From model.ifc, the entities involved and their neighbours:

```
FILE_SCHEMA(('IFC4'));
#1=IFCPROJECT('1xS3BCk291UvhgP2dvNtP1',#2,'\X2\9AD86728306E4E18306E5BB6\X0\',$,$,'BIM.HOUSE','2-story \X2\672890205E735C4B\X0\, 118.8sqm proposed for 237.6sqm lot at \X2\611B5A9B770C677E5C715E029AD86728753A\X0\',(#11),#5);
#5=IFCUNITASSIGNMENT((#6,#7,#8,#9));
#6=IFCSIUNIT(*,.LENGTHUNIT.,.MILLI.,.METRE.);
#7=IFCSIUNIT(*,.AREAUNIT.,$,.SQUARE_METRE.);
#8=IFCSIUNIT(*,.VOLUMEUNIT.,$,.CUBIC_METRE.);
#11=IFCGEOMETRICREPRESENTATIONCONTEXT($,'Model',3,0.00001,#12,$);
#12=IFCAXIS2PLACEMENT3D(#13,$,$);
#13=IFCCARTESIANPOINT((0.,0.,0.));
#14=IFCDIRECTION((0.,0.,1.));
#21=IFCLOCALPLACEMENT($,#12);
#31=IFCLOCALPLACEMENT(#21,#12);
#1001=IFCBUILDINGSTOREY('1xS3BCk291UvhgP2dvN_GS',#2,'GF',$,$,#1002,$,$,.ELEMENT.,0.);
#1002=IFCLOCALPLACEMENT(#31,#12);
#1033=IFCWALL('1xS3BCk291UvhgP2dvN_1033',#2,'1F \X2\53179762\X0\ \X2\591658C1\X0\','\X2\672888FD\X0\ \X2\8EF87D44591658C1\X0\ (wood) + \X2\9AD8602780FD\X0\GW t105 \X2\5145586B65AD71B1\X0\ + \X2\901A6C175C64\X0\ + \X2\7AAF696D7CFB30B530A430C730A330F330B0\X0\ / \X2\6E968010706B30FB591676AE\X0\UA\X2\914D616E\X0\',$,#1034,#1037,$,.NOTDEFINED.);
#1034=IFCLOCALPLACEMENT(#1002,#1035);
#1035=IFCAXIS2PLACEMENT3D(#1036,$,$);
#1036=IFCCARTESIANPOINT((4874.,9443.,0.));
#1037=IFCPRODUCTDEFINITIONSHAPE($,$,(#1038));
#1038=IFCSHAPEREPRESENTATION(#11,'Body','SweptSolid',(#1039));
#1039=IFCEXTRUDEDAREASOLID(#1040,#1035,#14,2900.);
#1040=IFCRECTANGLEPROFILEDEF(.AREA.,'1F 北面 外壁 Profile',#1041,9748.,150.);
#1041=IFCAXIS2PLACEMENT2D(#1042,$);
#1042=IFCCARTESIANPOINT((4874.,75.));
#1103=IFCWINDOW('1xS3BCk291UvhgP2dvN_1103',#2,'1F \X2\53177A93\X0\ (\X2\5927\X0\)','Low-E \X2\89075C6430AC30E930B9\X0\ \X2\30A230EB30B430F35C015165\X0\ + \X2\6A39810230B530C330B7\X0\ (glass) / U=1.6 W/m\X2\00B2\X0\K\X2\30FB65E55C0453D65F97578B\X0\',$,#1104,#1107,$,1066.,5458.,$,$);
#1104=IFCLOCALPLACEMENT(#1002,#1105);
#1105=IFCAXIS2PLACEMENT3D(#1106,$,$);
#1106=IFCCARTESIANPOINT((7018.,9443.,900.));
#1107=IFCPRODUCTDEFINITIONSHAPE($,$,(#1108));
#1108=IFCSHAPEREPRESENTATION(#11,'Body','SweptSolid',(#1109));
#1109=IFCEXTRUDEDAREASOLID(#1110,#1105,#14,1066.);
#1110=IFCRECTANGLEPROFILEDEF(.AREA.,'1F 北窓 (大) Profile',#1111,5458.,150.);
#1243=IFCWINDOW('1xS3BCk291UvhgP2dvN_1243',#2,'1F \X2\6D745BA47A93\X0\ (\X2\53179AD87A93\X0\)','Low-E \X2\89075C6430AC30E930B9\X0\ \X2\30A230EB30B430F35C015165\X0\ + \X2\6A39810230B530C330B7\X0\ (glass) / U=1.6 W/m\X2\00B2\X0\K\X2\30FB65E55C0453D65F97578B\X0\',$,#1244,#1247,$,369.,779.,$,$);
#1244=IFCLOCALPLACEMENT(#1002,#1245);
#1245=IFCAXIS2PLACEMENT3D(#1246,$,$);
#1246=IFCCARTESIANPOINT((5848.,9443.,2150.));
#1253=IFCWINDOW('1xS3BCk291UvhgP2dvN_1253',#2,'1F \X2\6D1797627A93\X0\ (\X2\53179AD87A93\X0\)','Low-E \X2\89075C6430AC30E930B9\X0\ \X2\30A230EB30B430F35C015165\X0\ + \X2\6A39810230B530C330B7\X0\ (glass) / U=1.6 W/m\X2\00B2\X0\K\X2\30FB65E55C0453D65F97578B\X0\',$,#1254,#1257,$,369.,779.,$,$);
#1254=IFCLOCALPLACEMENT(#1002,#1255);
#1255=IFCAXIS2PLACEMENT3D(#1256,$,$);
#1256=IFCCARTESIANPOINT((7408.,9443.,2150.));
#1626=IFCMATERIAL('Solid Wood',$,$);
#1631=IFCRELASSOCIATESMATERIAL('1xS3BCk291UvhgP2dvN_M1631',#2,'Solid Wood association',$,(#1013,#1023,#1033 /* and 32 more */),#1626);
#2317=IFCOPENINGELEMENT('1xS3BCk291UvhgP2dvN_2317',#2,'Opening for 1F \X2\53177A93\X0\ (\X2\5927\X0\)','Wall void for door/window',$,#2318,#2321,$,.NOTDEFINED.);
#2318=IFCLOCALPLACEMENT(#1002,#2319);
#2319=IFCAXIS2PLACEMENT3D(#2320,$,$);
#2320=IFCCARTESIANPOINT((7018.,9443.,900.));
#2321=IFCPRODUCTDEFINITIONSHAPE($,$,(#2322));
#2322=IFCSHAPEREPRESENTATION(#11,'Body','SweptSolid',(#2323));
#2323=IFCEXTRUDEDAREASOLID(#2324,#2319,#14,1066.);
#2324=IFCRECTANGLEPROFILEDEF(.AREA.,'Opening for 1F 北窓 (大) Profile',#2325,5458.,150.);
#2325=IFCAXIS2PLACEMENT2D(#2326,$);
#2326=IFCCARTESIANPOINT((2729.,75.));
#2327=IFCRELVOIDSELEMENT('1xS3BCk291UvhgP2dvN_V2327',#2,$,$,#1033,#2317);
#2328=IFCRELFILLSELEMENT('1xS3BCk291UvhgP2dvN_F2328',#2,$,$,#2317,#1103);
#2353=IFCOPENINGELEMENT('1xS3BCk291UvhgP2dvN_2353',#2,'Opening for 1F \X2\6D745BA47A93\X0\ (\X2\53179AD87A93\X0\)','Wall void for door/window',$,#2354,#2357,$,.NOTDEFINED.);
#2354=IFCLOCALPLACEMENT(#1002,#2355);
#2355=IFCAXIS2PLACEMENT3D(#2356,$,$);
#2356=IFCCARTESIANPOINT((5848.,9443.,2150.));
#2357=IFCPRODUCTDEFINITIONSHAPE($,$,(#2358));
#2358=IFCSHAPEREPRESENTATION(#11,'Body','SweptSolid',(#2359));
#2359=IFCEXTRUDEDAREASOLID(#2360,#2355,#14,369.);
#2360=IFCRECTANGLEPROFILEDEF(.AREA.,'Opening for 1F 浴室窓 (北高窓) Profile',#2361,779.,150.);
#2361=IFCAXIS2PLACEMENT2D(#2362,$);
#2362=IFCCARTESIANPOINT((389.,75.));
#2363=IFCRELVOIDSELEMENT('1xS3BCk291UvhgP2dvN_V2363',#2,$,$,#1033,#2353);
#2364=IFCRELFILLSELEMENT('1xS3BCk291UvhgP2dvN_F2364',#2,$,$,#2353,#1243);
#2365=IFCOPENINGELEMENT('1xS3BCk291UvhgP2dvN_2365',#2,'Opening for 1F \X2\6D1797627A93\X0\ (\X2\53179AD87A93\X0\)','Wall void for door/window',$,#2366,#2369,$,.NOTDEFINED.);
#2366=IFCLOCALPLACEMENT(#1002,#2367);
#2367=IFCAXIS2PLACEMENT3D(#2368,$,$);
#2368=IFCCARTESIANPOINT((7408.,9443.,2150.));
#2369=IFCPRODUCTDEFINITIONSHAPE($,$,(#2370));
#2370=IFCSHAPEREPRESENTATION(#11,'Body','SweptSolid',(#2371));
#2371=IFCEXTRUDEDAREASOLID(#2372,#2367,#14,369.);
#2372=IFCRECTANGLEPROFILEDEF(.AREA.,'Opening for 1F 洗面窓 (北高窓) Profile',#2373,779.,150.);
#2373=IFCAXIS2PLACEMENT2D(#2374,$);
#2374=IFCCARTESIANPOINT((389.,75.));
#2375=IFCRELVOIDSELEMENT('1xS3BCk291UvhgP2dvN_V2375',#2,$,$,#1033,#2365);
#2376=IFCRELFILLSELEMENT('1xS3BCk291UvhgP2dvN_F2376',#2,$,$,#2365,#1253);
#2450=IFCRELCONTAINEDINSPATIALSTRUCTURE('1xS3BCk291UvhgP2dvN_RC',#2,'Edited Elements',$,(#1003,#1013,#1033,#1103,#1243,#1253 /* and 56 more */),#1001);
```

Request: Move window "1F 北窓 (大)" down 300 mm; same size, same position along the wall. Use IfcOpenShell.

```python
import numpy as np
import ifcopenshell
import ifcopenshell.api.geometry
import ifcopenshell.util.placement
import ifcopenshell.util.unit

model = ifcopenshell.open("model.ifc")
unit_scale = ifcopenshell.util.unit.calculate_unit_scale(model)

window = model.by_guid("1xS3BCk291UvhgP2dvN_1103")
opening = window.FillsVoids[0].RelatingOpeningElement
dz = -0.3 / unit_scale

shift = np.array([0.0, 0.0, dz])
# The window is not placed relative to its opening, so move both.
for product in (opening, window):
    matrix = ifcopenshell.util.placement.get_local_placement(product.ObjectPlacement)
    matrix[:3, 3] += shift
    ifcopenshell.api.geometry.edit_object_placement(model, product=product, matrix=matrix, is_si=False)

print(f"moved by {dz * unit_scale:+.3f} m")

model.write("model_rev.ifc")
```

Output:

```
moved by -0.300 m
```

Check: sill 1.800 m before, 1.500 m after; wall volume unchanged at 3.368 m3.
